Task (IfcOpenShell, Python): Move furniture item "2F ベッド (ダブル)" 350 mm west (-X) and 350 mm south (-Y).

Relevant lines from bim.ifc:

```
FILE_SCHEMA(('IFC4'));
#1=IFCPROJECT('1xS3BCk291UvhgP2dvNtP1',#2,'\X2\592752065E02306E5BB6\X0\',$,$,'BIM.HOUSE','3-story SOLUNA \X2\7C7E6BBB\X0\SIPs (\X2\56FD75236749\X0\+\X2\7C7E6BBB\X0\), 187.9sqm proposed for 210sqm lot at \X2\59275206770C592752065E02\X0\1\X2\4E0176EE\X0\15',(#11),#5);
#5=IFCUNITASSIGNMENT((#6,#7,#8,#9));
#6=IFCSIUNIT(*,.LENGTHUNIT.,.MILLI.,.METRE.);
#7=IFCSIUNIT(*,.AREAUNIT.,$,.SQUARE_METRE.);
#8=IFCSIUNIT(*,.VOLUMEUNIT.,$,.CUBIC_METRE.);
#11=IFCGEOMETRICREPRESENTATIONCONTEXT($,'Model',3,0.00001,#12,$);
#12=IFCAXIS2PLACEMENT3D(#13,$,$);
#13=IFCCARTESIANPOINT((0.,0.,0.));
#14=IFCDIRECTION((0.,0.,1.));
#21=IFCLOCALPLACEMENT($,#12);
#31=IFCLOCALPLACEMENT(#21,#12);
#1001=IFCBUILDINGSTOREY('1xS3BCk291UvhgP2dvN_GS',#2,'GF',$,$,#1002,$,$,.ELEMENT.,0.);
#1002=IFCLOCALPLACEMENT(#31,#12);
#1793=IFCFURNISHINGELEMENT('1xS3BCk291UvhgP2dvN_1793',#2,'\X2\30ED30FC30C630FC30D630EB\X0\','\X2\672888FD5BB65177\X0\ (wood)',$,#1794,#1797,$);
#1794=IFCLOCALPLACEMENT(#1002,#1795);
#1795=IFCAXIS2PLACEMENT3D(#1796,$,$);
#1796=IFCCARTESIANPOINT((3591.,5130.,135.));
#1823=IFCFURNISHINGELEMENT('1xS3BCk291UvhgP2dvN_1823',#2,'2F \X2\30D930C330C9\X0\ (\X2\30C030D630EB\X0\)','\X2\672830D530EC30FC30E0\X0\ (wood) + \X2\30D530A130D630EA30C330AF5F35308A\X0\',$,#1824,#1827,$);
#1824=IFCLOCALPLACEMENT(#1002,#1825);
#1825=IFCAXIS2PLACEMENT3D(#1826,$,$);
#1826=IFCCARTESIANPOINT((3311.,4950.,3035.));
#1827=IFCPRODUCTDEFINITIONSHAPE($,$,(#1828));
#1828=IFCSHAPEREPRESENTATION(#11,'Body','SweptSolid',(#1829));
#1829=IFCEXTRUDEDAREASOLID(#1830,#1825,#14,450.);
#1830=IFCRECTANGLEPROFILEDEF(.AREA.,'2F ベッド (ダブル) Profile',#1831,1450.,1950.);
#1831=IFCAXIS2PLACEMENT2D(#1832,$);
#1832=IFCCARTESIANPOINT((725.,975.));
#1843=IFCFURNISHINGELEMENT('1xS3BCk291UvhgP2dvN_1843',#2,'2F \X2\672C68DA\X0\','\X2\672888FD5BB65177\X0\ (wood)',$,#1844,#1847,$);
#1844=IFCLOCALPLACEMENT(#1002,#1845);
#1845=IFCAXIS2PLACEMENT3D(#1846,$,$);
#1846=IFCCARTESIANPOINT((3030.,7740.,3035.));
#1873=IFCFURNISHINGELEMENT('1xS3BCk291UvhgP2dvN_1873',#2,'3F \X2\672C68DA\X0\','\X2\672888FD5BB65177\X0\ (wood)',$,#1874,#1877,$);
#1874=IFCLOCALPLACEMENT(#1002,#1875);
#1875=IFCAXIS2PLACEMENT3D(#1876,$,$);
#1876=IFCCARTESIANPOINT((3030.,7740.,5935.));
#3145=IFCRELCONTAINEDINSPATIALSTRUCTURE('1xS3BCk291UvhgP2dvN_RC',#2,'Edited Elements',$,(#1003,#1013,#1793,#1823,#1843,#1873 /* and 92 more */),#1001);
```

```python
import ifcopenshell
import ifcopenshell.api.geometry
import ifcopenshell.util.placement
import ifcopenshell.util.unit

model = ifcopenshell.open("bim.ifc")
unit_scale = ifcopenshell.util.unit.calculate_unit_scale(model)

item = model.by_guid("1xS3BCk291UvhgP2dvN_1823")
matrix = ifcopenshell.util.placement.get_local_placement(item.ObjectPlacement)
matrix[0, 3] -= 0.35 / unit_scale
matrix[1, 3] -= 0.35 / unit_scale
ifcopenshell.api.geometry.edit_object_placement(model, product=item, matrix=matrix, is_si=False)

print(ifcopenshell.util.placement.get_local_placement(item.ObjectPlacement).round(3) + 0.0)

model.write("bim-out.ifc")
```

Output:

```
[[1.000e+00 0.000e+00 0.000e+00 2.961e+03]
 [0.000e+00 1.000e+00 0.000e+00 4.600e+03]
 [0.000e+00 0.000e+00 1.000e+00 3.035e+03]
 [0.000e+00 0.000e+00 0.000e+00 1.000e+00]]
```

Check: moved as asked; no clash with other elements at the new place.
